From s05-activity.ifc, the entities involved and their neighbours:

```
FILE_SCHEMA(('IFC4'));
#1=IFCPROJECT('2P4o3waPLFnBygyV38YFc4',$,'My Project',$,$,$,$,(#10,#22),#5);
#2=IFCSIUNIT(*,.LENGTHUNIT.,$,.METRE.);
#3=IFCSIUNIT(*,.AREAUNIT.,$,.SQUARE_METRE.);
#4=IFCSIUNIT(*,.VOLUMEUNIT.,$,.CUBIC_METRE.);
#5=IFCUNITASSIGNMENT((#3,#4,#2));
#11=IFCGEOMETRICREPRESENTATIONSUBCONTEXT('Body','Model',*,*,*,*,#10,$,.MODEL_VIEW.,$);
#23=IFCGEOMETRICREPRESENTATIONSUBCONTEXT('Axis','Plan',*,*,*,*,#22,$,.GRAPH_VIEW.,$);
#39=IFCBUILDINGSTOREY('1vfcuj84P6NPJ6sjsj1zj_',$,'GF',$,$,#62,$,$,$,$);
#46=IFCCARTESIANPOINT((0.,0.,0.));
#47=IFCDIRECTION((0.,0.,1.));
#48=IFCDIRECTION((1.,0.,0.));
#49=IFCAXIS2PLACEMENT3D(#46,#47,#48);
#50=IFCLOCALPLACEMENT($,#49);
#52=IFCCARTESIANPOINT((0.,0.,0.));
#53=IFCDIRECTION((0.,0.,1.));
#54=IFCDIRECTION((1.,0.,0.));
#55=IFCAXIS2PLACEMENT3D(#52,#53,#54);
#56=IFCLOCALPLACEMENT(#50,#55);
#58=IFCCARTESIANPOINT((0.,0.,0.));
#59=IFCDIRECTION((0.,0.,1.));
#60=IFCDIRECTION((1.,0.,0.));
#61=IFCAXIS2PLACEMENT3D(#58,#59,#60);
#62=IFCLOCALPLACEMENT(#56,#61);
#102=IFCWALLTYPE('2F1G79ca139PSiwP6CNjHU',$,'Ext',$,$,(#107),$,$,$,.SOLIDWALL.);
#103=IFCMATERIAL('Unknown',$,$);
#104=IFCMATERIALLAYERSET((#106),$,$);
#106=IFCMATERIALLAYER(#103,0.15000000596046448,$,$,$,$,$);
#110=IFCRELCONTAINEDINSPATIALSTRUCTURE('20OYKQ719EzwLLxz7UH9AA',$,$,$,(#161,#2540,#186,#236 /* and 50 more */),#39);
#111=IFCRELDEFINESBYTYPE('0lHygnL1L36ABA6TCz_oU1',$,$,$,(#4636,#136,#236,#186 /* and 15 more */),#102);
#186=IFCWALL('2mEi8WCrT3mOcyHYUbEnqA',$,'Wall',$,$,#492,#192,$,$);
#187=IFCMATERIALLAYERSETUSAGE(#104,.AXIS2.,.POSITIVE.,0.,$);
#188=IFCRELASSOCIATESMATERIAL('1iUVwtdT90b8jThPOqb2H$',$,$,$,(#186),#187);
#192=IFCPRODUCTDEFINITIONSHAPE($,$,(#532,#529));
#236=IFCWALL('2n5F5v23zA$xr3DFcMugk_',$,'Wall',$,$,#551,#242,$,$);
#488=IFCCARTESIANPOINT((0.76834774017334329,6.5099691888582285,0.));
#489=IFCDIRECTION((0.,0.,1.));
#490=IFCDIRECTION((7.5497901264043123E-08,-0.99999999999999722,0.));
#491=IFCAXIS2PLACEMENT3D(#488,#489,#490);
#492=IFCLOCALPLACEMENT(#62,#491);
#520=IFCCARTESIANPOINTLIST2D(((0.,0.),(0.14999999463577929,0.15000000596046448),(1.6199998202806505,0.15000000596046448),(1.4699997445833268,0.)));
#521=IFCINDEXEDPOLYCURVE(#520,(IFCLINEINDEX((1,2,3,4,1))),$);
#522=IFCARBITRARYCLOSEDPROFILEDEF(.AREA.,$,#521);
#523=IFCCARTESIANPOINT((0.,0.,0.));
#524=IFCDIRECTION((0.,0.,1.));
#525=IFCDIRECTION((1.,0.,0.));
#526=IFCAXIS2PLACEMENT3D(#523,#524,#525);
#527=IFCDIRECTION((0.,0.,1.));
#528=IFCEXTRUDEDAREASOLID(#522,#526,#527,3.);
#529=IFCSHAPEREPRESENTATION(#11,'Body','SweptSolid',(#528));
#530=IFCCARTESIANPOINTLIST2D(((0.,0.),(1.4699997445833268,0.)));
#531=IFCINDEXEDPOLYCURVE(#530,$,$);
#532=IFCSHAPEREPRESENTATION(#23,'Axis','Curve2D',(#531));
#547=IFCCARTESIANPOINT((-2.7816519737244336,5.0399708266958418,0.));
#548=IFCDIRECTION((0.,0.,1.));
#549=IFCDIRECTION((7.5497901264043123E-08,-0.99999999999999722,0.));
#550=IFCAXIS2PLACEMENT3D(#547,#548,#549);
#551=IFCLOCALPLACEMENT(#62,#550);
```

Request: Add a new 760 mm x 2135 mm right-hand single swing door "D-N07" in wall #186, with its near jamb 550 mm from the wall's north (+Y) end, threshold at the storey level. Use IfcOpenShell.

```python
import numpy as np
import ifcopenshell
import ifcopenshell.api.feature
import ifcopenshell.api.geometry
import ifcopenshell.api.root
import ifcopenshell.api.spatial
import ifcopenshell.geom
import ifcopenshell.util.element
import ifcopenshell.util.placement
import ifcopenshell.util.representation
import ifcopenshell.util.shape
import ifcopenshell.util.unit

model = ifcopenshell.open("s05-activity.ifc")
unit_scale = ifcopenshell.util.unit.calculate_unit_scale(model)
settings = ifcopenshell.geom.settings()


def volume(element):
    """Net volume in cubic metres, openings subtracted."""
    shape = ifcopenshell.geom.create_shape(settings, element)
    return ifcopenshell.util.shape.get_volume(shape.geometry)


wall = model.by_id(186)
storey = ifcopenshell.util.element.get_container(wall, ifc_class="IfcBuildingStorey")
context = ifcopenshell.util.representation.get_context(model, "Model", "Body", "MODEL_VIEW")
before = volume(wall)

width, height, from_end, sill = 0.76, 2.135, 0.55, 0.0  # metres

# The wall runs along its own X axis, and the end named is its -X end.
wall_shape = ifcopenshell.geom.create_shape(settings, wall)
x, y, z = ifcopenshell.util.shape.get_vertices(wall_shape.geometry).T
start = x.min() + from_end
face, thickness = float(y.min()), float(y.max() - y.min())
wall_matrix = ifcopenshell.util.placement.get_local_placement(wall.ObjectPlacement)
level = ifcopenshell.util.placement.get_local_placement(storey.ObjectPlacement)[2, 3]


def in_wall(x, y):
    """Placement at x, y metres in the wall's axes, at sill height."""
    matrix = wall_matrix.copy()
    matrix[:, 3] = wall_matrix @ np.array([x / unit_scale, y / unit_scale, 0.0, 1.0])
    matrix[2, 3] = level + sill / unit_scale
    return matrix


# Opening: a box that overshoots both wall faces by 50 mm.
opening = ifcopenshell.api.root.create_entity(model, ifc_class="IfcOpeningElement", predefined_type="OPENING")
box = ifcopenshell.api.geometry.add_wall_representation(
    model, context=context, length=width, height=height, thickness=thickness + 0.1
)
ifcopenshell.api.geometry.assign_representation(model, product=opening, representation=box)
ifcopenshell.api.geometry.edit_object_placement(model, product=opening, matrix=in_wall(start, face - 0.05), is_si=False)
ifcopenshell.api.feature.add_feature(model, feature=opening, element=wall)

door = ifcopenshell.api.root.create_entity(model, ifc_class="IfcDoor", name="D-N07", predefined_type="DOOR")
door.OverallWidth, door.OverallHeight = width / unit_scale, height / unit_scale
door.OperationType = "SINGLE_SWING_RIGHT"
body = ifcopenshell.api.geometry.add_door_representation(
    model,
    context=context,
    overall_width=door.OverallWidth,
    overall_height=door.OverallHeight,
    operation_type="SINGLE_SWING_RIGHT",
    lining_properties={"LiningDepth": thickness / unit_scale, "ThresholdDepth": thickness / unit_scale},
)
ifcopenshell.api.geometry.assign_representation(model, product=door, representation=body)
ifcopenshell.api.spatial.assign_container(model, products=[door], relating_structure=storey)
ifcopenshell.api.feature.add_filling(model, opening=opening, element=door)

# The lining spans the wall, so the door starts at the wall face.
ifcopenshell.api.geometry.edit_object_placement(model, product=door, matrix=in_wall(start, face), is_si=False)

after = volume(wall)

print(f"wall volume {before:.3f} -> {after:.3f} m3")

model.write("s05-activity_edited.ifc")
```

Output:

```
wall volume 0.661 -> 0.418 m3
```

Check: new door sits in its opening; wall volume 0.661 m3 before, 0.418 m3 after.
